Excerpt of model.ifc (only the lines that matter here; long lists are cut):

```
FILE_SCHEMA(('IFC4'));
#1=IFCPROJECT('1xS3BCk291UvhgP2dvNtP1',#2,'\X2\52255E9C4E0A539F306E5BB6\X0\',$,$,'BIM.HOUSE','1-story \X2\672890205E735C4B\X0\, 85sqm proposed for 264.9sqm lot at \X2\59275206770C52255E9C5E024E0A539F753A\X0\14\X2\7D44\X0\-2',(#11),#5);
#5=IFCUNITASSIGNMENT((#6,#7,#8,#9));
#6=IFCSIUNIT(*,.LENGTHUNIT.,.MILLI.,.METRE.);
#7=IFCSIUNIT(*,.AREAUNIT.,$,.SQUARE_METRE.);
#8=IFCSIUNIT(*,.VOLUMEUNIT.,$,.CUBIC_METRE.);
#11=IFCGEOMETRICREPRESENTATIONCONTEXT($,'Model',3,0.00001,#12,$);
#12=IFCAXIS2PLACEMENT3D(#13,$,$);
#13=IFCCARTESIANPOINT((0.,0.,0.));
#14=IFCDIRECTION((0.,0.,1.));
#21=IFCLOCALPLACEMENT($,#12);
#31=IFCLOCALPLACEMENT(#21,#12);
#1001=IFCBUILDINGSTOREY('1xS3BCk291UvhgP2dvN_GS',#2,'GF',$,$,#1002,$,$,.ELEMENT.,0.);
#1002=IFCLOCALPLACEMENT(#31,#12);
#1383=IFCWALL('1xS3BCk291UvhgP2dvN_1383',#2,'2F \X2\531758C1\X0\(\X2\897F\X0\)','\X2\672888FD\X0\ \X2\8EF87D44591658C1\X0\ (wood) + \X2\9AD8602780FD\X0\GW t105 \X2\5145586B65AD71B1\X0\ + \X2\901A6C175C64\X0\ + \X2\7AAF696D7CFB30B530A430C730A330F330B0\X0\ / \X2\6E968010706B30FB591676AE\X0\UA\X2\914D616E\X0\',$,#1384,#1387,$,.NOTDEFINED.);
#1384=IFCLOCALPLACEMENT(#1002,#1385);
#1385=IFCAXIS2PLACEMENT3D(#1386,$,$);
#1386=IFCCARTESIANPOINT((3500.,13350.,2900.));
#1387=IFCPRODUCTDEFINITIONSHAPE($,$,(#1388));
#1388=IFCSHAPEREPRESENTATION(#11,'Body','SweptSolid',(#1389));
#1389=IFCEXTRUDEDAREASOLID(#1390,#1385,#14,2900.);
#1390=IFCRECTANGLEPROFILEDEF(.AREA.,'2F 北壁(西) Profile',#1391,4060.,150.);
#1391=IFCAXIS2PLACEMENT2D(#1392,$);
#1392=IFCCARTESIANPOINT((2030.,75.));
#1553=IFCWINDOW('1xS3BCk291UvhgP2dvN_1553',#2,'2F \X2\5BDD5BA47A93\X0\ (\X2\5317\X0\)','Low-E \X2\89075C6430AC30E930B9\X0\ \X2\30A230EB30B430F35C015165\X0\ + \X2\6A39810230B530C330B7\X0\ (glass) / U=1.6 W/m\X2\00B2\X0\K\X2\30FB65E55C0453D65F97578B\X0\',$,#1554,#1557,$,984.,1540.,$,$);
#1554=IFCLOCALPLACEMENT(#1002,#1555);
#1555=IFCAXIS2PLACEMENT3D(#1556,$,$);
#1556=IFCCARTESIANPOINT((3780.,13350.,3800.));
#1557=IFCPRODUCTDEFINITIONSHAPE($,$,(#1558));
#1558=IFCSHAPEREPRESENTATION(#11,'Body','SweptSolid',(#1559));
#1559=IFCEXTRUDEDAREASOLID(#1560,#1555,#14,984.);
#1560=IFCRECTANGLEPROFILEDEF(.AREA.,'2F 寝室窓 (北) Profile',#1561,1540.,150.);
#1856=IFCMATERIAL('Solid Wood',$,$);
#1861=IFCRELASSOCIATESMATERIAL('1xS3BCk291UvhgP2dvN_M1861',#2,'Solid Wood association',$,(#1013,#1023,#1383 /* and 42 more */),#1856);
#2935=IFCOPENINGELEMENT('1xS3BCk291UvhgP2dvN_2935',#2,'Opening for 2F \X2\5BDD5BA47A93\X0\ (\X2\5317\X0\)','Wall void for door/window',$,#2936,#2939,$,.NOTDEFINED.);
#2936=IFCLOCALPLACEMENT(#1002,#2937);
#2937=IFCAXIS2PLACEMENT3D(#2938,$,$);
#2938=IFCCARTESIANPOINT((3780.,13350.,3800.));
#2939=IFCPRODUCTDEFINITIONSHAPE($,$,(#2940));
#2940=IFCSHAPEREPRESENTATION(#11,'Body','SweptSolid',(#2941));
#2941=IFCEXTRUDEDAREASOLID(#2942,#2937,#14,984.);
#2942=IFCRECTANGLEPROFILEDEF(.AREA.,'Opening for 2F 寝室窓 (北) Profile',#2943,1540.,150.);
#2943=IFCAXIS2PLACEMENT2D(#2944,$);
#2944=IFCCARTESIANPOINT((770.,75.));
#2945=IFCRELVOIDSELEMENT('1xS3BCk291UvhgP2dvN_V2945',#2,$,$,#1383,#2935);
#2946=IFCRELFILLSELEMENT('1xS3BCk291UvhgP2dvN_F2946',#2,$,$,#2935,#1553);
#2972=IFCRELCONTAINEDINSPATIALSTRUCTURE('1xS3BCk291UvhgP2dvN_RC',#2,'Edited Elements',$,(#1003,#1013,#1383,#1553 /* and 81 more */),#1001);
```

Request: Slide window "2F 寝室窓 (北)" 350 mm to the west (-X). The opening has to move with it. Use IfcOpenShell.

```python
import ifcopenshell
import ifcopenshell.api.geometry
import ifcopenshell.util.placement
import ifcopenshell.util.unit

model = ifcopenshell.open("model.ifc")
unit_scale = ifcopenshell.util.unit.calculate_unit_scale(model)

window = model.by_guid("1xS3BCk291UvhgP2dvN_1553")
opening = window.FillsVoids[0].RelatingOpeningElement
wall = opening.VoidsElements[0].RelatingBuildingElement

wall_matrix = ifcopenshell.util.placement.get_local_placement(wall.ObjectPlacement)
shift = wall_matrix[:3, 0] * -0.35 / unit_scale
before = ifcopenshell.util.placement.get_local_placement(window.ObjectPlacement)[:3, 3].copy()

# The window is not placed relative to its opening, so move both.
for product in (opening, window):
    matrix = ifcopenshell.util.placement.get_local_placement(product.ObjectPlacement)
    matrix[:3, 3] += shift
    ifcopenshell.api.geometry.edit_object_placement(model, product=product, matrix=matrix, is_si=False)

after = ifcopenshell.util.placement.get_local_placement(window.ObjectPlacement)[:3, 3]
print("window moved by", (after - before).round(3) + 0.0)

model.write("model-out.ifc")
```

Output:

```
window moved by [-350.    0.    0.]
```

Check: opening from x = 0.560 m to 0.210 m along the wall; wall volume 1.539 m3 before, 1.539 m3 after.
